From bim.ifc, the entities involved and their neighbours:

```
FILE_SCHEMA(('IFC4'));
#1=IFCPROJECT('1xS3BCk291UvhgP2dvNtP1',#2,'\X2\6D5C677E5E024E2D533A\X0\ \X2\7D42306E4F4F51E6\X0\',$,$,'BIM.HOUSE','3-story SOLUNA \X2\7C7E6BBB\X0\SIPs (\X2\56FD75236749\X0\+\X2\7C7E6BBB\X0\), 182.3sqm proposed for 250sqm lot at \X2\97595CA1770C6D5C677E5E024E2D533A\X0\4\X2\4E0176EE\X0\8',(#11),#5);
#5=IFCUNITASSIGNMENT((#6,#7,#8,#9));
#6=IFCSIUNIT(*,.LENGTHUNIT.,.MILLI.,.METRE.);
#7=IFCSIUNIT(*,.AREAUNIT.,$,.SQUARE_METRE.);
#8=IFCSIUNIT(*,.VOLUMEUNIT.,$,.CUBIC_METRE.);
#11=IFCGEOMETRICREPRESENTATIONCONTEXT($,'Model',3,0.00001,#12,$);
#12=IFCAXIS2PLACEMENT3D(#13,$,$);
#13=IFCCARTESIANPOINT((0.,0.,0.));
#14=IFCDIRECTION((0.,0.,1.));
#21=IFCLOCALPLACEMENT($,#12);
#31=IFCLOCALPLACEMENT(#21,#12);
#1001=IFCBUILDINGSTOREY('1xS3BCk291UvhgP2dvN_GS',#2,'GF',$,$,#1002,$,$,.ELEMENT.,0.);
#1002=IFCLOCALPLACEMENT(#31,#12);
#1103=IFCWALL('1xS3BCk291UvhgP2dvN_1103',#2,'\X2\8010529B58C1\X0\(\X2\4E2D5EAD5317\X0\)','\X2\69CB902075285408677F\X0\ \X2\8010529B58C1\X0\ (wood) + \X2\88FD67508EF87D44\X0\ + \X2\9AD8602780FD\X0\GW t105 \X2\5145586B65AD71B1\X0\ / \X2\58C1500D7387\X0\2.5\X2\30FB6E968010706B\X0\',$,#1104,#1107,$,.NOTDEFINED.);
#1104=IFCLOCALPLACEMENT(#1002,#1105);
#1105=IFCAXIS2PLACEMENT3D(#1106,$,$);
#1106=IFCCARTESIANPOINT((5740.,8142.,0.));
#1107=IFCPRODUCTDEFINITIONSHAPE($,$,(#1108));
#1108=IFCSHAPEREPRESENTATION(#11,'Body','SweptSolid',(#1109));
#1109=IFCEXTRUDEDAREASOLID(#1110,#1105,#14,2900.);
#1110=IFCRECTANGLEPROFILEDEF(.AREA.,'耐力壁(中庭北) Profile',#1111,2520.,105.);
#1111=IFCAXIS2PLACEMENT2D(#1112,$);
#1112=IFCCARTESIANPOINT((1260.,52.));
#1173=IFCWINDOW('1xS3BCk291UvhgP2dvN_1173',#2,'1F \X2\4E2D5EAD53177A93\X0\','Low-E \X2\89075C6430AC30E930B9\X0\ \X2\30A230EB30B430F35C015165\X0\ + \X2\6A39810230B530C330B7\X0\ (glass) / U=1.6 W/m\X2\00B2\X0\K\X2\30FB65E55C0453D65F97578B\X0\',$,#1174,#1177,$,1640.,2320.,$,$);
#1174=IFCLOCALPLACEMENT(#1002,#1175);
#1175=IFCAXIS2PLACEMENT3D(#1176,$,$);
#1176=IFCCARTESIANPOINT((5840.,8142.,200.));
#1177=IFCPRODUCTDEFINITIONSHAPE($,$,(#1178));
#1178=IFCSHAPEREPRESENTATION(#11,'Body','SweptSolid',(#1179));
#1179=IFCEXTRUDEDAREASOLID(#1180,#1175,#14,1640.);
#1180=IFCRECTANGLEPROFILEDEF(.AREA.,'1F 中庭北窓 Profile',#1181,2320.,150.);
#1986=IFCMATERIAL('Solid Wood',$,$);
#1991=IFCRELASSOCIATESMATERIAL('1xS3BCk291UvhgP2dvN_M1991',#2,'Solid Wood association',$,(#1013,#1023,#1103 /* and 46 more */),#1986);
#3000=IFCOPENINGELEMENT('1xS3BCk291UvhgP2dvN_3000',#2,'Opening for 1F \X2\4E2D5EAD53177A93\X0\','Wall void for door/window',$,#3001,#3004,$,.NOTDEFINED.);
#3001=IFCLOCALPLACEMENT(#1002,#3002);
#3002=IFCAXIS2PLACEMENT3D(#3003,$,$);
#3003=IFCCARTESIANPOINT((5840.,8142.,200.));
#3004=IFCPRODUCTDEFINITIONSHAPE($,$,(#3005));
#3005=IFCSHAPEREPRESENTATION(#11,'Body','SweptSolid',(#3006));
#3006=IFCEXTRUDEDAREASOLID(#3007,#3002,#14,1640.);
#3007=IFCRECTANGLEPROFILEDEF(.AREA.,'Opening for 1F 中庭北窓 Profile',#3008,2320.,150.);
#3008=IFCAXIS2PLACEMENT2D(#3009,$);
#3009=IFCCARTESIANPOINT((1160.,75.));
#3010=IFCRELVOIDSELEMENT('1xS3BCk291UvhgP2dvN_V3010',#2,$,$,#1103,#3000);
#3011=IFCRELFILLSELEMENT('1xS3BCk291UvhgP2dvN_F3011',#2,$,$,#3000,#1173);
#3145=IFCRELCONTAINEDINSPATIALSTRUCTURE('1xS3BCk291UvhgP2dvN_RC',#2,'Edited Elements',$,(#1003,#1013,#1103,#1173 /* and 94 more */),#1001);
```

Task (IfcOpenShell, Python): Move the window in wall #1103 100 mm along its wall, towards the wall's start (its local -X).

```python
import ifcopenshell
import ifcopenshell.api.geometry
import ifcopenshell.util.placement
import ifcopenshell.util.unit

model = ifcopenshell.open("bim.ifc")
unit_scale = ifcopenshell.util.unit.calculate_unit_scale(model)

window = model.by_guid("1xS3BCk291UvhgP2dvN_1173")
opening = window.FillsVoids[0].RelatingOpeningElement
wall = opening.VoidsElements[0].RelatingBuildingElement

wall_matrix = ifcopenshell.util.placement.get_local_placement(wall.ObjectPlacement)
shift = wall_matrix[:3, 0] * -0.1 / unit_scale
before = ifcopenshell.util.placement.get_local_placement(window.ObjectPlacement)[:3, 3].copy()

# The window is not placed relative to its opening, so move both.
for product in (opening, window):
    matrix = ifcopenshell.util.placement.get_local_placement(product.ObjectPlacement)
    matrix[:3, 3] += shift
    ifcopenshell.api.geometry.edit_object_placement(model, product=product, matrix=matrix, is_si=False)

after = ifcopenshell.util.placement.get_local_placement(window.ObjectPlacement)[:3, 3]
print("window moved by", (after - before).round(3) + 0.0)

model.write("bim_v2.ifc")
```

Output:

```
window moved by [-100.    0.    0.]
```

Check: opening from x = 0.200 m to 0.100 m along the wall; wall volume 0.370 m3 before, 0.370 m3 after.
